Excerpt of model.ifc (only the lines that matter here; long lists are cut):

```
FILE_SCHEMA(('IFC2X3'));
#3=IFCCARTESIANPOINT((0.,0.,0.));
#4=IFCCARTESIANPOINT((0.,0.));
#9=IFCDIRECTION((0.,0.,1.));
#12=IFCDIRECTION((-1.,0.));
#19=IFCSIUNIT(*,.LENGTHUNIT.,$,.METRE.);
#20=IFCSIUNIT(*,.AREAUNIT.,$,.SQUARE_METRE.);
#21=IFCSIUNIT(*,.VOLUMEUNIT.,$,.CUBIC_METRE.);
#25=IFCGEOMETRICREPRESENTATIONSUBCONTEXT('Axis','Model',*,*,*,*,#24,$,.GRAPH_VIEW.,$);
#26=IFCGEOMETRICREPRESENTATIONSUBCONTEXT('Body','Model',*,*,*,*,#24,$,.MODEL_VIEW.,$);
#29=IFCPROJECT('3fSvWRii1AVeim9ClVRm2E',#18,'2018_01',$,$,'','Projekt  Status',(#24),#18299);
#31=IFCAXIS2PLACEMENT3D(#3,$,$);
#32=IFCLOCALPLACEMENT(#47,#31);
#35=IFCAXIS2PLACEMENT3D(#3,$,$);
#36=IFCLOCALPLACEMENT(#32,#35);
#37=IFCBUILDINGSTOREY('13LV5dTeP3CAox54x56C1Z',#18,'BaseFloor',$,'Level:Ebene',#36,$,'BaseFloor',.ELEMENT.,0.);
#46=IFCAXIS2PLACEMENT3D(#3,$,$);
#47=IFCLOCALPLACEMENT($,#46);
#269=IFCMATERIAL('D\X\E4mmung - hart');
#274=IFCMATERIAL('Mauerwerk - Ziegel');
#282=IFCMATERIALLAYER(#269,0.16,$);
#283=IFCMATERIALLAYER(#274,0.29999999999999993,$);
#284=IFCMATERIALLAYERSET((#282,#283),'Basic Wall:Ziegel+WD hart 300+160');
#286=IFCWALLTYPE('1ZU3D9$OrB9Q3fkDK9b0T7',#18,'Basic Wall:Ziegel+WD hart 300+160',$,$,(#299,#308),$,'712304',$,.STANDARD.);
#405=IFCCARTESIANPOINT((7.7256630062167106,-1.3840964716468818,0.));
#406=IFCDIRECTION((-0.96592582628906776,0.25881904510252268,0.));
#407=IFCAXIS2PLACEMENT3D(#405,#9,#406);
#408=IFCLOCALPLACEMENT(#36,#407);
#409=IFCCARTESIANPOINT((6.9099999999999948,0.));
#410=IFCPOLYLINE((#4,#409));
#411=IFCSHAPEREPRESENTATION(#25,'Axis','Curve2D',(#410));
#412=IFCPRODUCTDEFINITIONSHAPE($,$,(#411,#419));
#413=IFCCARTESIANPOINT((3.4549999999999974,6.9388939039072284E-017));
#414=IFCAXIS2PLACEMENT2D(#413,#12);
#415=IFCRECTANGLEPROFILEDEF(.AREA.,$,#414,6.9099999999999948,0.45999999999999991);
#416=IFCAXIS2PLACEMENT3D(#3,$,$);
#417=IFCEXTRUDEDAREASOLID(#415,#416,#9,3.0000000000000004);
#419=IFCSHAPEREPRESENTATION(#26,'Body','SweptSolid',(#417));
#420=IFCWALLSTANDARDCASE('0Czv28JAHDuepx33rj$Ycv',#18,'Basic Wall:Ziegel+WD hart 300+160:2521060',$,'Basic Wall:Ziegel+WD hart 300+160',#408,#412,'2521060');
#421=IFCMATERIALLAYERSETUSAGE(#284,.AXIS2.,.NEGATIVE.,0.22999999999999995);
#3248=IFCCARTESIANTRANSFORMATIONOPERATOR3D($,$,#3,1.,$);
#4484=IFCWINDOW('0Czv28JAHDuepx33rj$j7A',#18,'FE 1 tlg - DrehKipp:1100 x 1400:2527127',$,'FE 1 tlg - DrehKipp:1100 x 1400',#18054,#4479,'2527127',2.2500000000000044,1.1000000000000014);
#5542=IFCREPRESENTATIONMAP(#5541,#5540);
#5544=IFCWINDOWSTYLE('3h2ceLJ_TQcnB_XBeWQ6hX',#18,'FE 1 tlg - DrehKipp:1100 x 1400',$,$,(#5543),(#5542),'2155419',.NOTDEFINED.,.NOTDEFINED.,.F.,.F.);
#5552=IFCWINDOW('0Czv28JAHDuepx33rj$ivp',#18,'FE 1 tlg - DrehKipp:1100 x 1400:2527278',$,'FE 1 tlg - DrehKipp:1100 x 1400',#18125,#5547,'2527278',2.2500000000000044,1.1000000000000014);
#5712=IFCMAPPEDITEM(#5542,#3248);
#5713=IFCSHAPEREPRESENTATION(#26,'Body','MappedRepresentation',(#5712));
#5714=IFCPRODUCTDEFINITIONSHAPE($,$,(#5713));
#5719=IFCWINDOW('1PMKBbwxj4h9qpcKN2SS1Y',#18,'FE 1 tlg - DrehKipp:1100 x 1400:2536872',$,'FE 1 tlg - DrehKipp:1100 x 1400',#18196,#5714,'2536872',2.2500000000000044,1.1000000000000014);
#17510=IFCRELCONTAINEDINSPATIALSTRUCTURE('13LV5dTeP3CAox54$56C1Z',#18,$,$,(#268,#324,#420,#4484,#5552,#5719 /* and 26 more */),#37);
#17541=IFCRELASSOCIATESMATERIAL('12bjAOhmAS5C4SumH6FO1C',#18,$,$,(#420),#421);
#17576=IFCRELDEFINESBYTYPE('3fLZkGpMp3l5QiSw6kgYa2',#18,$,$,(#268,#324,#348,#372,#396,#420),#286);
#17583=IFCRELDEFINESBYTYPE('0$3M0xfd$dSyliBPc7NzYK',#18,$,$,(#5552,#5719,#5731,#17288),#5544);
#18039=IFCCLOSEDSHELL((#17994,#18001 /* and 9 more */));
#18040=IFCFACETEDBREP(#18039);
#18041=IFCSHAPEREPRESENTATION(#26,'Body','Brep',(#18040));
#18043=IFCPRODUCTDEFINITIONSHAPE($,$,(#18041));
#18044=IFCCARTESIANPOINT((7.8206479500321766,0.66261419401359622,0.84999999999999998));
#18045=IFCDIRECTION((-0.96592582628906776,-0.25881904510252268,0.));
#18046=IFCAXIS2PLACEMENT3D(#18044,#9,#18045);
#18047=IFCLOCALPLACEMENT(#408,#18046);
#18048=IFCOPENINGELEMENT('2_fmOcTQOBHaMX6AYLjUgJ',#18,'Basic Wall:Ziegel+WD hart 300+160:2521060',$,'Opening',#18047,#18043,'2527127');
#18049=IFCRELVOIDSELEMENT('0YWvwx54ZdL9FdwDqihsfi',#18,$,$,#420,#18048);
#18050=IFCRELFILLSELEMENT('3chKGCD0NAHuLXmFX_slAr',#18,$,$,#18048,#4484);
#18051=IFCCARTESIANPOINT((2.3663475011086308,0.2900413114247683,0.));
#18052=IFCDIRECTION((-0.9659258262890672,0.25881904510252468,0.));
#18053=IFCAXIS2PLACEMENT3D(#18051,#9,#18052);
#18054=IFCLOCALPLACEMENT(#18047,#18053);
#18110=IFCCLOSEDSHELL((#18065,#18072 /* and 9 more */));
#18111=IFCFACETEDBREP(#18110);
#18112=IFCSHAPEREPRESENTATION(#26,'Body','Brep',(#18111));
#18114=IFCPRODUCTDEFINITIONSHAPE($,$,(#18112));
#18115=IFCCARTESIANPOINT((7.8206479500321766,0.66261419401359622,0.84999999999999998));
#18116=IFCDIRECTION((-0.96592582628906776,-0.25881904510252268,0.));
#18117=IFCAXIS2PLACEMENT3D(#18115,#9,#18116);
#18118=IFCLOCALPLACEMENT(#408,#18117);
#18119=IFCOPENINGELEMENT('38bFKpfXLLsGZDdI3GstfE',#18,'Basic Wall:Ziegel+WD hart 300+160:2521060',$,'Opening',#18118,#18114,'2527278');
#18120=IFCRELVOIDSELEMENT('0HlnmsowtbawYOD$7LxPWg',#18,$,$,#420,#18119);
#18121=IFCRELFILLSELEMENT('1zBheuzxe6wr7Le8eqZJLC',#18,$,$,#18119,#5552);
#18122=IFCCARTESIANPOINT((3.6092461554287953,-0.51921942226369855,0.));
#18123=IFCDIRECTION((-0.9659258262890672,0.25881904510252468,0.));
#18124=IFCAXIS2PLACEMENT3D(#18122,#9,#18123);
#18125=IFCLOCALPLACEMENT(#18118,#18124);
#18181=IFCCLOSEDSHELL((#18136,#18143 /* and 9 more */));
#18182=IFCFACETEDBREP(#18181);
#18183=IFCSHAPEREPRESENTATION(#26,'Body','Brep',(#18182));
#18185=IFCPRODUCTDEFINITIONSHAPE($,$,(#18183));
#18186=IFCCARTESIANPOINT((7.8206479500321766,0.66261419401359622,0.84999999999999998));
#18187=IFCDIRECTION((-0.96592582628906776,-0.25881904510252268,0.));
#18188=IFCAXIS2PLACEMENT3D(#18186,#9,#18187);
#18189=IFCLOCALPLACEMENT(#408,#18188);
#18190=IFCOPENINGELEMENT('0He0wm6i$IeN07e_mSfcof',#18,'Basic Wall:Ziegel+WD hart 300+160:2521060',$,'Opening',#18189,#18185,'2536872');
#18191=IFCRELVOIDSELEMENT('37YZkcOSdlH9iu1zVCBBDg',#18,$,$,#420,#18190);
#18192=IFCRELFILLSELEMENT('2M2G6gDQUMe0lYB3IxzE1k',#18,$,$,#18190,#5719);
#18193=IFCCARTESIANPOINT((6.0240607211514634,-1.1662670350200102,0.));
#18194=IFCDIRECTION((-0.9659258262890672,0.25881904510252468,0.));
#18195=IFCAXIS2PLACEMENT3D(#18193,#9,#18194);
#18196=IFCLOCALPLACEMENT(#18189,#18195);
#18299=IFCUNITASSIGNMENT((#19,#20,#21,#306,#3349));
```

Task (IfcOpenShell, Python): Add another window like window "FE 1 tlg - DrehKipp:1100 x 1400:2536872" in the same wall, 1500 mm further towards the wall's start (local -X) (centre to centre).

```python
import ifcopenshell
import ifcopenshell.api.feature
import ifcopenshell.api.geometry
import ifcopenshell.api.root
import ifcopenshell.geom
import ifcopenshell.util.element
import ifcopenshell.util.placement
import ifcopenshell.util.shape

model = ifcopenshell.open("model.ifc")
settings = ifcopenshell.geom.settings()


def volume(element):
    """Net volume in cubic metres, openings subtracted."""
    shape = ifcopenshell.geom.create_shape(settings, element)
    return ifcopenshell.util.shape.get_volume(shape.geometry)


def reuse_history(source, copy):
    """copy_class also copies each property set's owner history, people and application; keep the originals."""
    for rel in copy.IsDefinedBy:
        if rel.is_a("IfcRelDefinesByProperties") and (history := rel.RelatingPropertyDefinition.OwnerHistory):
            rel.RelatingPropertyDefinition.OwnerHistory = source.OwnerHistory
            ifcopenshell.util.element.remove_deep2(model, history)


window = model.by_guid("1PMKBbwxj4h9qpcKN2SS1Y")
opening = window.FillsVoids[0].RelatingOpeningElement
wall = opening.VoidsElements[0].RelatingBuildingElement
before = volume(wall)
shift = ifcopenshell.util.placement.get_local_placement(wall.ObjectPlacement)[:3, 0] * -1.5

# copy_class copies the void relationship, type, container and properties, but no geometry.
new_opening = ifcopenshell.api.root.copy_class(model, product=opening)
new_opening.Representation = ifcopenshell.util.element.copy_deep(
    model, opening.Representation, exclude=["IfcGeometricRepresentationContext", "IfcRepresentationMap"]
)
new_opening.Name = "Basic Wall:Ziegel+WD hart 300+160"
new_opening.Tag = None
new_window = ifcopenshell.api.root.copy_class(model, product=window)
new_window.Representation = ifcopenshell.util.element.copy_deep(
    model, window.Representation, exclude=["IfcGeometricRepresentationContext", "IfcRepresentationMap"]
)
new_window.Name = "FE 1 tlg - DrehKipp:1100 x 1400"
new_window.Tag = None
reuse_history(window, new_window)
fills = ifcopenshell.api.feature.add_filling(model, opening=new_opening, element=new_window)
fills.OwnerHistory = new_window.OwnerHistory  # required in IFC2X3

for old, new in ((opening, new_opening), (window, new_window)):
    matrix = ifcopenshell.util.placement.get_local_placement(old.ObjectPlacement)
    matrix[:3, 3] += shift
    ifcopenshell.api.geometry.edit_object_placement(model, product=new, matrix=matrix, is_si=False)

after = volume(wall)

print(f"wall volume {before:.3f} -> {after:.3f} m3")

model.write("model-out.ifc")
```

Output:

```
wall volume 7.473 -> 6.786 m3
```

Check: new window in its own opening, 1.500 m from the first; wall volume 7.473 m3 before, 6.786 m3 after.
